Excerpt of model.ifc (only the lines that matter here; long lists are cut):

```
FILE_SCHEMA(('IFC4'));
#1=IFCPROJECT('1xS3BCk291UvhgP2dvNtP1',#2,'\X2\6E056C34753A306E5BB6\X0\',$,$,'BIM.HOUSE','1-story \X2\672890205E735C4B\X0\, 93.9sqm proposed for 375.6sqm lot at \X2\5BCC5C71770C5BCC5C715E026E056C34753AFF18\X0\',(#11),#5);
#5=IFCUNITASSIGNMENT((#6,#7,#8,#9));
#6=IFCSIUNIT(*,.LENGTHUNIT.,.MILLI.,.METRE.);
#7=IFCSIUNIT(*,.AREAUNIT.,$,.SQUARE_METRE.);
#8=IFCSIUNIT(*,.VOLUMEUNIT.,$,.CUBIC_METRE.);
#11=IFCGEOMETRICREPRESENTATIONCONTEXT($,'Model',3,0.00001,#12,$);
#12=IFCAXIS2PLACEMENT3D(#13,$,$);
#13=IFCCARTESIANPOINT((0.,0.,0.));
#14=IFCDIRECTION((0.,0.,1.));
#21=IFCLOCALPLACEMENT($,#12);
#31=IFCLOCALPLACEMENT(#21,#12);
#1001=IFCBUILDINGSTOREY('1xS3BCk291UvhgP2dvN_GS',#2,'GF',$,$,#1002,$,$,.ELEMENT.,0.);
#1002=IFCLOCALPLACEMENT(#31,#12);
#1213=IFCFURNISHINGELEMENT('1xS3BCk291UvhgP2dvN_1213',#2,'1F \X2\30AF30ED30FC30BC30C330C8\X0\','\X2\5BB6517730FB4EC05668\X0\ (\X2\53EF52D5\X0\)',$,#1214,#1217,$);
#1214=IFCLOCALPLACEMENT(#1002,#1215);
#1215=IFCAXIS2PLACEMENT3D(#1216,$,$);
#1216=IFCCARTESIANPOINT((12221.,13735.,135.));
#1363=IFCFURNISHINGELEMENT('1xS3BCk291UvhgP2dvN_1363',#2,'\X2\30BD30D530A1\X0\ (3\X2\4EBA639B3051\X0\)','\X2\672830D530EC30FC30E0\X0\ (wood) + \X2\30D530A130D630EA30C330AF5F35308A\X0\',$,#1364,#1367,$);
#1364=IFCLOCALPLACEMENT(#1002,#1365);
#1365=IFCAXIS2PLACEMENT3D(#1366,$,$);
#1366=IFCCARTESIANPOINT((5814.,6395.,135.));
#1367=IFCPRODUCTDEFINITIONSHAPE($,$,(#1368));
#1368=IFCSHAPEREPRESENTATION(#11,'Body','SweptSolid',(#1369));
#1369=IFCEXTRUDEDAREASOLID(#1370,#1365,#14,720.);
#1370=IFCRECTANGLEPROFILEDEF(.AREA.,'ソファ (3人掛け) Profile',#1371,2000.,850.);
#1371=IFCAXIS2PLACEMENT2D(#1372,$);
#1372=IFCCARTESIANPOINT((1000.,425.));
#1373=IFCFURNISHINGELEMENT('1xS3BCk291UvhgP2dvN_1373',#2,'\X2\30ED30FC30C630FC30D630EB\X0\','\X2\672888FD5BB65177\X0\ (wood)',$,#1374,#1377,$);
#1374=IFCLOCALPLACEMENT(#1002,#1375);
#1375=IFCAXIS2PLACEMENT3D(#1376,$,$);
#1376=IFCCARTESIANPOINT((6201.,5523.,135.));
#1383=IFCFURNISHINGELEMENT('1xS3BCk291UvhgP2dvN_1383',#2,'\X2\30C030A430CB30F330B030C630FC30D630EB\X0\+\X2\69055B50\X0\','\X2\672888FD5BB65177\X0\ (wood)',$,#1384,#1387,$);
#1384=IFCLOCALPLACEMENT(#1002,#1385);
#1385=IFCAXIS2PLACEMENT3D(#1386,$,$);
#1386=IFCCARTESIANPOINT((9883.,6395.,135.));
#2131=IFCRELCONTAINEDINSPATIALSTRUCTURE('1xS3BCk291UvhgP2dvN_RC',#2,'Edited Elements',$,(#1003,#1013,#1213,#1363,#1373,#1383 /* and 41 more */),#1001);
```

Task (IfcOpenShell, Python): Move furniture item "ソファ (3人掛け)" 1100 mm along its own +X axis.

```python
import ifcopenshell
import ifcopenshell.api.geometry
import ifcopenshell.util.placement
import ifcopenshell.util.unit

model = ifcopenshell.open("model.ifc")
unit_scale = ifcopenshell.util.unit.calculate_unit_scale(model)

item = model.by_guid("1xS3BCk291UvhgP2dvN_1363")
matrix = ifcopenshell.util.placement.get_local_placement(item.ObjectPlacement)
matrix[:3, 3] += matrix[:3, 0] * 1.1 / unit_scale
ifcopenshell.api.geometry.edit_object_placement(model, product=item, matrix=matrix, is_si=False)

print(ifcopenshell.util.placement.get_local_placement(item.ObjectPlacement).round(3) + 0.0)

model.write("model_updated.ifc")
```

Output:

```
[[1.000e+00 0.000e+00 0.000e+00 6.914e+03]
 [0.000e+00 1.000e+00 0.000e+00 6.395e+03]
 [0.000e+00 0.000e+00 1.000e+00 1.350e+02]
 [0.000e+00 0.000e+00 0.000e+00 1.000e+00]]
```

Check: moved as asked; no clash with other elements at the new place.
